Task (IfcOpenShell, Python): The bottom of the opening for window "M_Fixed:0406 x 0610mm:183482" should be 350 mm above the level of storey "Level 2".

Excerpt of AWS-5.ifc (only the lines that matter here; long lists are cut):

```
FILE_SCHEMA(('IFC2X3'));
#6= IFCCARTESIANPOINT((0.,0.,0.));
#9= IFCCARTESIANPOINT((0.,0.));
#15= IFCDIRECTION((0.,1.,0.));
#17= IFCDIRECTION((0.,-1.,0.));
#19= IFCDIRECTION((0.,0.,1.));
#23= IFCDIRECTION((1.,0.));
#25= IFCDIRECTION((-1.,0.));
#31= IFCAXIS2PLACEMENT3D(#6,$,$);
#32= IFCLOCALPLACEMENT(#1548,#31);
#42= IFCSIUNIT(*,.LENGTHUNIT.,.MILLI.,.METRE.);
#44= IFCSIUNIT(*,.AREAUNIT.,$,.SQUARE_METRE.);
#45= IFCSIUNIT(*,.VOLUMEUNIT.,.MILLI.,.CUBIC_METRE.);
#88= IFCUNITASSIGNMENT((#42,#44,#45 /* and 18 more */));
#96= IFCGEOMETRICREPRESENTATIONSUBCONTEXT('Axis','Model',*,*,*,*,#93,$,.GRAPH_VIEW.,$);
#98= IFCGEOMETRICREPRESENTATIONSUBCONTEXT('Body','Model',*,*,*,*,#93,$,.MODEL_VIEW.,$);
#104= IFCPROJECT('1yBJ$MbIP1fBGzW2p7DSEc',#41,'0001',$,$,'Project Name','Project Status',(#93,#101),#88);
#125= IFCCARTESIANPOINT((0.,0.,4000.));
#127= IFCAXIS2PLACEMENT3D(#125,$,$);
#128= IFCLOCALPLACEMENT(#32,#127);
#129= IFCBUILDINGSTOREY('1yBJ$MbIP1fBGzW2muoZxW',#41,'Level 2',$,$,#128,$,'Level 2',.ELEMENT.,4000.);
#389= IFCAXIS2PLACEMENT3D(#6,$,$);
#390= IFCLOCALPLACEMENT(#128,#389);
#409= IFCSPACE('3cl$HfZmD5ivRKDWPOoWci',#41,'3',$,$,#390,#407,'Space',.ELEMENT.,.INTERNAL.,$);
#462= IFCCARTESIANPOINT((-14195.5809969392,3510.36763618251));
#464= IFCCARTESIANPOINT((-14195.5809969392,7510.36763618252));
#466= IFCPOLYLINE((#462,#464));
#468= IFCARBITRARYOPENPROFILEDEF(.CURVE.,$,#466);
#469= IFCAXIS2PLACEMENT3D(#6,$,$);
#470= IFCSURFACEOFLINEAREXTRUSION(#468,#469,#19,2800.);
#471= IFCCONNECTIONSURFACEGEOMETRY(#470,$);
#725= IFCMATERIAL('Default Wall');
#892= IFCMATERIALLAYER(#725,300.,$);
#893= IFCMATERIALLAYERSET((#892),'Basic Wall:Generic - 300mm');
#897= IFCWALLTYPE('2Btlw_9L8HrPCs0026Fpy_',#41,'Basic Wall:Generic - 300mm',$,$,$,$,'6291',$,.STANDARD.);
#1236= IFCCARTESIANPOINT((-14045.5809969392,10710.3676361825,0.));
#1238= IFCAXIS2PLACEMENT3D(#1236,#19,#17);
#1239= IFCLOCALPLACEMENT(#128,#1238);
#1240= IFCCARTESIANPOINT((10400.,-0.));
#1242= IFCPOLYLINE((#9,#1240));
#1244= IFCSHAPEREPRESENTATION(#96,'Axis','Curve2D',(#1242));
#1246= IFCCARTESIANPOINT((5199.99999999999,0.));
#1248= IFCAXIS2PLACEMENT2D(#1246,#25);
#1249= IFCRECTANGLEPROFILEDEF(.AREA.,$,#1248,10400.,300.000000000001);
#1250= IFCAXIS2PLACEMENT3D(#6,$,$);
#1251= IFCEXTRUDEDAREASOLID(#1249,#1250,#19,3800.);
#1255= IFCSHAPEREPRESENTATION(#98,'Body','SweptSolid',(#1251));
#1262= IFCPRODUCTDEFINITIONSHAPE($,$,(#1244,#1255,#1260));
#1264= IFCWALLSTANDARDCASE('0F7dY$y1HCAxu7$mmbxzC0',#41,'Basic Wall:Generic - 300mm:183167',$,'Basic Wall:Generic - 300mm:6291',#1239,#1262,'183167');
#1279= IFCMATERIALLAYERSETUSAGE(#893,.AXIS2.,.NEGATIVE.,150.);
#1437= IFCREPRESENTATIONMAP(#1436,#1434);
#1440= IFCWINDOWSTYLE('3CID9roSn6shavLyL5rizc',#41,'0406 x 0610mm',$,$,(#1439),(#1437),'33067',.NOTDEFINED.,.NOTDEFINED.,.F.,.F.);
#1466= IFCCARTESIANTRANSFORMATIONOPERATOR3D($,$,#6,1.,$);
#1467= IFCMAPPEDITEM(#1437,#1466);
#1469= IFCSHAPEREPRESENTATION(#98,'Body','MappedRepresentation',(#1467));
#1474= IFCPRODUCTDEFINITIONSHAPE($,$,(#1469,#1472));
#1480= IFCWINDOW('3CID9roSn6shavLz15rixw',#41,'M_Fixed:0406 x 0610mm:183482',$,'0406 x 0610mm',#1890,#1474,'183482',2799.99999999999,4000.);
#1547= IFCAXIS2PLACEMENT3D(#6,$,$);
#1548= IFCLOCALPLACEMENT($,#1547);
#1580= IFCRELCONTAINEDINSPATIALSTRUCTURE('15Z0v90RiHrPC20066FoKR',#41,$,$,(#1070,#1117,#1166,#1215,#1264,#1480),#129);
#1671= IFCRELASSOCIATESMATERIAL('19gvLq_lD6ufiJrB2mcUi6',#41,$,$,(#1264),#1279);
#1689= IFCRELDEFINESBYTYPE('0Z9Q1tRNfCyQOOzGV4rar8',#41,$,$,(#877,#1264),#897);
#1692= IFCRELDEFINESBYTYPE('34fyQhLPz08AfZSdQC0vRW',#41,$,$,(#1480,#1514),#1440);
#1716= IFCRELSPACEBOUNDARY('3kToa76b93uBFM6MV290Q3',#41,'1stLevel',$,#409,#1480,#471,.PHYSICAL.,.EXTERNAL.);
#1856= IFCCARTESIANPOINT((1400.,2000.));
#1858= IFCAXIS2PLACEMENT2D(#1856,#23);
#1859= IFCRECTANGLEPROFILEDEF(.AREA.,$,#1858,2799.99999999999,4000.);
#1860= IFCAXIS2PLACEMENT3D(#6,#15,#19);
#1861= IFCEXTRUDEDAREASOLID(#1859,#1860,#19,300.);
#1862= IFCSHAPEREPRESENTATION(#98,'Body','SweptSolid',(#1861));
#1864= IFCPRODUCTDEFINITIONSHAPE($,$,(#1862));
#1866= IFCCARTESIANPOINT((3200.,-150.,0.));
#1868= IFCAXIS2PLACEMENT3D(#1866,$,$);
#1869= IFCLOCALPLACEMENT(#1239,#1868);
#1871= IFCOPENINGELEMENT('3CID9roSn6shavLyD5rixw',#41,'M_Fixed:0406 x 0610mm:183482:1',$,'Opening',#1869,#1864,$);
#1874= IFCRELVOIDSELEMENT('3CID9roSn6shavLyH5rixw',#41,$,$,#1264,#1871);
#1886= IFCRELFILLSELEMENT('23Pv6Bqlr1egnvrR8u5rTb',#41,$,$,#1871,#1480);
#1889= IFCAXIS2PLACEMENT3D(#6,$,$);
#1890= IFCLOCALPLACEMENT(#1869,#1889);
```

```python
import numpy as np
import ifcopenshell
import ifcopenshell.api.geometry
import ifcopenshell.geom
import ifcopenshell.util.element
import ifcopenshell.util.placement
import ifcopenshell.util.shape
import ifcopenshell.util.unit

model = ifcopenshell.open("AWS-5.ifc")
unit_scale = ifcopenshell.util.unit.calculate_unit_scale(model)

window = model.by_guid("3CID9roSn6shavLz15rixw")
opening = window.FillsVoids[0].RelatingOpeningElement
storey = ifcopenshell.util.element.get_container(window, ifc_class="IfcBuildingStorey")
level = ifcopenshell.util.placement.get_local_placement(storey.ObjectPlacement)[2, 3]

# The opening's origin need not be at the sill, so measure its lowest point.
shape = ifcopenshell.geom.create_shape(ifcopenshell.geom.settings(), opening)
bottom = ifcopenshell.util.shape.get_shape_bottom_elevation(shape, shape.geometry) / unit_scale
dz = level + 0.35 / unit_scale - bottom

shift = np.array([0.0, 0.0, dz])
# The window is placed relative to its opening, so it follows when the opening moves.
matrix = ifcopenshell.util.placement.get_local_placement(opening.ObjectPlacement)
matrix[:3, 3] += shift
ifcopenshell.api.geometry.edit_object_placement(
    model, product=opening, matrix=matrix, is_si=False, should_transform_children=True
)

# Space boundary surfaces are stored in each space's coordinates; move them too.
for rel in window.ProvidesBoundaries:
    if not rel.ConnectionGeometry:
        continue
    surface = rel.ConnectionGeometry.SurfaceOnRelatingElement
    space_matrix = ifcopenshell.util.placement.get_local_placement(rel.RelatingSpace.ObjectPlacement)
    point = np.array(surface.Position.Location.Coordinates) + space_matrix[:3, :3].T @ shift
    surface.Position = model.createIfcAxis2Placement3D(
        model.createIfcCartesianPoint(point.tolist()), surface.Position.Axis, surface.Position.RefDirection
    )

print(f"moved by {dz * unit_scale:+.3f} m")

model.write("AWS-5_updated.ifc")
```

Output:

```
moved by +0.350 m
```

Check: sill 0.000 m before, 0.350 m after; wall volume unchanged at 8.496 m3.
